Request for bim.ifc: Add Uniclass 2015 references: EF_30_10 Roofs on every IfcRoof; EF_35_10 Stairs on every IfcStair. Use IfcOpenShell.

First a look at what the model holds.

```python
import ifcopenshell

model = ifcopenshell.open("bim.ifc")
print(model.schema)
print("classifications:", [c.Name for c in model.by_type("IfcClassification")])
for ifc_class in ("IfcDoor", "IfcRoof", "IfcStair", "IfcWall", "IfcWindow"):
    print(ifc_class, len(model.by_type(ifc_class)))
```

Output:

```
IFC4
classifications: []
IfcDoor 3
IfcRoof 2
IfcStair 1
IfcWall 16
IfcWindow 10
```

```python
import ifcopenshell
import ifcopenshell.api.classification

model = ifcopenshell.open("bim.ifc")

system = ifcopenshell.api.classification.add_classification(model, classification="Uniclass 2015")

codes = {
    "IfcRoof": ("EF_30_10", "Roofs"),
    "IfcStair": ("EF_35_10", "Stairs"),
}
for ifc_class, (code, name) in codes.items():
    products = model.by_type(ifc_class)
    ifcopenshell.api.classification.add_reference(
        model, products=products, classification=system, identification=code, name=name
    )
    print(code, len(products))

model.write("bim-out.ifc")
```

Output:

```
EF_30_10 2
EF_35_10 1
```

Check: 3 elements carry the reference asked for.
